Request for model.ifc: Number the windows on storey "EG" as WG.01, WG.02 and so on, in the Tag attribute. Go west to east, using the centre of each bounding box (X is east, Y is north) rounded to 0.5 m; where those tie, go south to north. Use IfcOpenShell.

First a look at what the model holds.

```python
import ifcopenshell
import ifcopenshell.util.element
import ifcopenshell.util.placement

model = ifcopenshell.open("model.ifc")
print(model.schema)
storey = next(s for s in model.by_type("IfcBuildingStorey") if s.Name == "EG")
windows = [e for e in ifcopenshell.util.element.get_decomposition(storey) if e.is_a("IfcWindow")]
for e in sorted(windows, key=lambda e: e.id()):
    origin = ifcopenshell.util.placement.get_local_placement(e.ObjectPlacement)[:3, 3]
    print(e.id(), e.Tag, e.Name, origin.round(2) + 0.0, sep=" | ")
```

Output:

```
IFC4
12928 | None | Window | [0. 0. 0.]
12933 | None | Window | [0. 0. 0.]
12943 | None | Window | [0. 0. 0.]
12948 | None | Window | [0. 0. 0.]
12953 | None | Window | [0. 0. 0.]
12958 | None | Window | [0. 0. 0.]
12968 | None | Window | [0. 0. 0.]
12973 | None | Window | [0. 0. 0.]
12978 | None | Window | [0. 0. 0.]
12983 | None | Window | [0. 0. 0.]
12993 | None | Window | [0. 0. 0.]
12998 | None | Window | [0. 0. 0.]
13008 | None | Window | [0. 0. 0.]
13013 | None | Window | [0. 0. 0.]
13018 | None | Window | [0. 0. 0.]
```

```python
import ifcopenshell
import ifcopenshell.geom
import ifcopenshell.util.element
import ifcopenshell.util.shape

model = ifcopenshell.open("model.ifc")
settings = ifcopenshell.geom.settings()
settings.set("use-world-coords", True)


def centre(element):
    shape = ifcopenshell.geom.create_shape(settings, element)
    return ifcopenshell.util.shape.get_bbox_centroid(shape.geometry)


storey = next(s for s in model.by_type("IfcBuildingStorey") if s.Name == "EG")
windows = [e for e in ifcopenshell.util.element.get_decomposition(storey) if e.is_a("IfcWindow")]

# Insertion points can sit at a corner or the storey origin, so sort by the geometry (in metres).
centres = {e: centre(e) for e in windows}
windows.sort(key=lambda e: (round(centres[e][0] / 0.5), centres[e][1]))

for i, e in enumerate(windows, start=1):
    number = f"WG.{i:02d}"
    e.Tag = number
    print(e.id(), number)

model.write("model_rev.ifc")
```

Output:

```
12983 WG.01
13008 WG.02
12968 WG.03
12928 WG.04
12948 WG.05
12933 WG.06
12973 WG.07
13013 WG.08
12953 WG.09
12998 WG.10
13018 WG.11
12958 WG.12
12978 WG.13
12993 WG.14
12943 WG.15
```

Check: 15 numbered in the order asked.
